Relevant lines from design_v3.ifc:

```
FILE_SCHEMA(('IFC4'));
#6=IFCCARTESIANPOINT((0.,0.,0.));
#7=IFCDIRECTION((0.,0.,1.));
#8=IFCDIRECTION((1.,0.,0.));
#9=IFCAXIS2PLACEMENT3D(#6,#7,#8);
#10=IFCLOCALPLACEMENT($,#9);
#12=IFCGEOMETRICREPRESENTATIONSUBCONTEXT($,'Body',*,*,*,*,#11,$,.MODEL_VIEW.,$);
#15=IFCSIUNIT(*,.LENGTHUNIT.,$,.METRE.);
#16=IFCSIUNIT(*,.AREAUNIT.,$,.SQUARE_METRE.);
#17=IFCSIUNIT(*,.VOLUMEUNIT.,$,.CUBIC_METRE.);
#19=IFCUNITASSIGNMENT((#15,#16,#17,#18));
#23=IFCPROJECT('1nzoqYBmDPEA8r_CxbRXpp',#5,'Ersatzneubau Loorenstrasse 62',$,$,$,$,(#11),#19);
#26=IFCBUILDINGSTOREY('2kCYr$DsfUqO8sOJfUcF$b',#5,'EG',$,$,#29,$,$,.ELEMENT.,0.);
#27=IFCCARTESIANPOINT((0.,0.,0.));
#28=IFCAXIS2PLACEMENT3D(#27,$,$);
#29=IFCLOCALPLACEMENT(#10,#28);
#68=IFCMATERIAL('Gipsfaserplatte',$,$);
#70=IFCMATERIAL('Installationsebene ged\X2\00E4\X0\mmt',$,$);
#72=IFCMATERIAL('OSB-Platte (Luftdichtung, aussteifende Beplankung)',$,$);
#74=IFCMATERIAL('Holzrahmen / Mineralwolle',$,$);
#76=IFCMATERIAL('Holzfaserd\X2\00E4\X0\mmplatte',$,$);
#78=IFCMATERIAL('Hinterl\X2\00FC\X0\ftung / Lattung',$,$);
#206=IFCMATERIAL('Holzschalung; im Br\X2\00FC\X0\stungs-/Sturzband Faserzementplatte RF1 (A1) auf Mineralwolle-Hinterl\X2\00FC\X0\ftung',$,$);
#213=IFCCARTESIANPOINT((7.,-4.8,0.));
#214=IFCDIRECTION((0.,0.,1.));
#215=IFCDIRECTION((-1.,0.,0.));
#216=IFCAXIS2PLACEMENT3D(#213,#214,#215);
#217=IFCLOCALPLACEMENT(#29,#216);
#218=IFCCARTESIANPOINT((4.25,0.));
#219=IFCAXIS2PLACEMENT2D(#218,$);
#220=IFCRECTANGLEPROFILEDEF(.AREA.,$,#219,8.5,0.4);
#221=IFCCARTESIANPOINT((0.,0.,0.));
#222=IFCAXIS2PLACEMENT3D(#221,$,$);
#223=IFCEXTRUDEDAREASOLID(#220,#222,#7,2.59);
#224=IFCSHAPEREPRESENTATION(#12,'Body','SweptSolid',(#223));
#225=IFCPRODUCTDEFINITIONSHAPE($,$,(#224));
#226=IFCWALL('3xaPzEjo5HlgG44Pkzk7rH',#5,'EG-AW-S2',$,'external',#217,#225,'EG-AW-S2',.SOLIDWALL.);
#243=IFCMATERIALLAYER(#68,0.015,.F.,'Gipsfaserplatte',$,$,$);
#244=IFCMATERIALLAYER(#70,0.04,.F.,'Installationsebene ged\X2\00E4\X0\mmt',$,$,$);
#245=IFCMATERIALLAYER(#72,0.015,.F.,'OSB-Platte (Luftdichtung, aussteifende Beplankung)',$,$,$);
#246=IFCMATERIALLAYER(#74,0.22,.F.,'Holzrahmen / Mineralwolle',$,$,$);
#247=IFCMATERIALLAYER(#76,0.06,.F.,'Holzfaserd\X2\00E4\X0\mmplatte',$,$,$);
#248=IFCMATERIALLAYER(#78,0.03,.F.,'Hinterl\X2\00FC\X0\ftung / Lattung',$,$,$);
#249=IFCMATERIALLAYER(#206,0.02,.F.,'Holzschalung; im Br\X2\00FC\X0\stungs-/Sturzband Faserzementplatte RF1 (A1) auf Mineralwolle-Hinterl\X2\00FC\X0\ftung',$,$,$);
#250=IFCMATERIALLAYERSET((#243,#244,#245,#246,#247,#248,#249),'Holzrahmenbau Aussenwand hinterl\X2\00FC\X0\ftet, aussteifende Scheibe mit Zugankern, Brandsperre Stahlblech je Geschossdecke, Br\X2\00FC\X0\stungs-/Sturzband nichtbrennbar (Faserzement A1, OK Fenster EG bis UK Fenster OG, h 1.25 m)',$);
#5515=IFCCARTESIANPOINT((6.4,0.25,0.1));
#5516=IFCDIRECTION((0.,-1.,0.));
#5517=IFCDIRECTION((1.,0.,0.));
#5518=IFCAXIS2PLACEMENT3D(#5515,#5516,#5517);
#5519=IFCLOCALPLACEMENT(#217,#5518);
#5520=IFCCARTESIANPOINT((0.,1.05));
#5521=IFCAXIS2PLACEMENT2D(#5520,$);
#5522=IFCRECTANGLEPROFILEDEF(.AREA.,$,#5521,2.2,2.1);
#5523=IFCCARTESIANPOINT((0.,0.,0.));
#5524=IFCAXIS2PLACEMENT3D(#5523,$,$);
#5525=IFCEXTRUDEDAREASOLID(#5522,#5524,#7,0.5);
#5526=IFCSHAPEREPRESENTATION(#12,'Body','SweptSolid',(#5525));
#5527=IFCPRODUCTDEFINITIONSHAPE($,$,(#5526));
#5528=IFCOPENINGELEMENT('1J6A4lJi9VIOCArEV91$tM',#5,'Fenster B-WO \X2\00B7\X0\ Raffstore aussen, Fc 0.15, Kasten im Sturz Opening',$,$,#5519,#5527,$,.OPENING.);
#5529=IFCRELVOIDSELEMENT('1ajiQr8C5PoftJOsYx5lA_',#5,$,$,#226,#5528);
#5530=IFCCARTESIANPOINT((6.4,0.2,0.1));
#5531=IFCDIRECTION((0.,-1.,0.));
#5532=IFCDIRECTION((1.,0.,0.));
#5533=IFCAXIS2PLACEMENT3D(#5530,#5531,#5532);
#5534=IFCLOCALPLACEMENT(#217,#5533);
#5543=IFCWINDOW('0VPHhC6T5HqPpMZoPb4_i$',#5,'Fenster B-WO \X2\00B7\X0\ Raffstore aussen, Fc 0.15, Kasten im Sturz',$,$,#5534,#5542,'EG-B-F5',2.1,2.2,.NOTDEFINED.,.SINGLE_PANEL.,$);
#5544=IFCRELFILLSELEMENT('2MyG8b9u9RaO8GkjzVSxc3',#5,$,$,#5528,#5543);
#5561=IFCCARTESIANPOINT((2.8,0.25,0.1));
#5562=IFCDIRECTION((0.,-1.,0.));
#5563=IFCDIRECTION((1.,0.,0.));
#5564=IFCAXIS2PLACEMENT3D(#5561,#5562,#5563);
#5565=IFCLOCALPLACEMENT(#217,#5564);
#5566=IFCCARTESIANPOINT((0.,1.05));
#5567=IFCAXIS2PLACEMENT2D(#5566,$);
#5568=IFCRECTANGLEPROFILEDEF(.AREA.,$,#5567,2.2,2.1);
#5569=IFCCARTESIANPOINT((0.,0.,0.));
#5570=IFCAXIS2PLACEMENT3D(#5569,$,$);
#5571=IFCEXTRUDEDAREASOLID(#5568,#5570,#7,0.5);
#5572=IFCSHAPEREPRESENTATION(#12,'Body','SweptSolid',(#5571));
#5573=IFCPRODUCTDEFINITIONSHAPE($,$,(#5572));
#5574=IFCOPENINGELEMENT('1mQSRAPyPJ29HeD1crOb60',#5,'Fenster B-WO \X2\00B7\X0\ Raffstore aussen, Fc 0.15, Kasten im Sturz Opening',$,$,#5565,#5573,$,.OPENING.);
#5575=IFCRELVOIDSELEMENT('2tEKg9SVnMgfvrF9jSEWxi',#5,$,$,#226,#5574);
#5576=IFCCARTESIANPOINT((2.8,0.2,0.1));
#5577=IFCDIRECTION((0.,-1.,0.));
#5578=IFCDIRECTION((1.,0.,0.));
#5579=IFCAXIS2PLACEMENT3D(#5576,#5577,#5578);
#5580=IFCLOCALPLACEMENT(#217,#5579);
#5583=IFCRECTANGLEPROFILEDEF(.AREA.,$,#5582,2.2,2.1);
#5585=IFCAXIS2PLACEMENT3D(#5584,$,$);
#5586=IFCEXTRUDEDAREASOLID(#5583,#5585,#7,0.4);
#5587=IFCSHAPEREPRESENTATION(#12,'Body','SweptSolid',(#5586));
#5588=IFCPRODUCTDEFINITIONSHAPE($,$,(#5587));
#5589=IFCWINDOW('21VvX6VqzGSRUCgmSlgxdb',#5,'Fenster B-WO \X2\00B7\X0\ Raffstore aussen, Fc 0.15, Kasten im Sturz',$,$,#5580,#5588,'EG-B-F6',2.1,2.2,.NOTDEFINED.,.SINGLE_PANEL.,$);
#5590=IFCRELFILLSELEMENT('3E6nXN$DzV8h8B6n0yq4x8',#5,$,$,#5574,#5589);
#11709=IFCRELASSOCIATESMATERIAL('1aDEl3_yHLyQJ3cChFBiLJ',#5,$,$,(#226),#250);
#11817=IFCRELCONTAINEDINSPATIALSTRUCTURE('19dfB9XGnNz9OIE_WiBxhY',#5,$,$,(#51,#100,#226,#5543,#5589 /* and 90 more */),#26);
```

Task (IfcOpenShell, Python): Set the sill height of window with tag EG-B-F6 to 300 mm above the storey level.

```python
import numpy as np
import ifcopenshell
import ifcopenshell.api.geometry
import ifcopenshell.geom
import ifcopenshell.util.element
import ifcopenshell.util.placement
import ifcopenshell.util.shape
import ifcopenshell.util.unit

model = ifcopenshell.open("design_v3.ifc")
unit_scale = ifcopenshell.util.unit.calculate_unit_scale(model)

window = model.by_id(5589)
opening = window.FillsVoids[0].RelatingOpeningElement
storey = ifcopenshell.util.element.get_container(window, ifc_class="IfcBuildingStorey")
level = ifcopenshell.util.placement.get_local_placement(storey.ObjectPlacement)[2, 3]

# The opening's origin need not be at the sill, so measure its lowest point.
shape = ifcopenshell.geom.create_shape(ifcopenshell.geom.settings(), opening)
bottom = ifcopenshell.util.shape.get_shape_bottom_elevation(shape, shape.geometry) / unit_scale
dz = level + 0.3 - bottom

shift = np.array([0.0, 0.0, dz])
# The window is not placed relative to its opening, so move both.
for product in (opening, window):
    matrix = ifcopenshell.util.placement.get_local_placement(product.ObjectPlacement)
    matrix[:3, 3] += shift
    ifcopenshell.api.geometry.edit_object_placement(model, product=product, matrix=matrix, is_si=False)

print(f"moved by {dz * unit_scale:+.3f} m")

model.write("design_v3_v2.ifc")
```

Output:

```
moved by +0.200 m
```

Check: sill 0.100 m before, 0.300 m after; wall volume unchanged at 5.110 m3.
